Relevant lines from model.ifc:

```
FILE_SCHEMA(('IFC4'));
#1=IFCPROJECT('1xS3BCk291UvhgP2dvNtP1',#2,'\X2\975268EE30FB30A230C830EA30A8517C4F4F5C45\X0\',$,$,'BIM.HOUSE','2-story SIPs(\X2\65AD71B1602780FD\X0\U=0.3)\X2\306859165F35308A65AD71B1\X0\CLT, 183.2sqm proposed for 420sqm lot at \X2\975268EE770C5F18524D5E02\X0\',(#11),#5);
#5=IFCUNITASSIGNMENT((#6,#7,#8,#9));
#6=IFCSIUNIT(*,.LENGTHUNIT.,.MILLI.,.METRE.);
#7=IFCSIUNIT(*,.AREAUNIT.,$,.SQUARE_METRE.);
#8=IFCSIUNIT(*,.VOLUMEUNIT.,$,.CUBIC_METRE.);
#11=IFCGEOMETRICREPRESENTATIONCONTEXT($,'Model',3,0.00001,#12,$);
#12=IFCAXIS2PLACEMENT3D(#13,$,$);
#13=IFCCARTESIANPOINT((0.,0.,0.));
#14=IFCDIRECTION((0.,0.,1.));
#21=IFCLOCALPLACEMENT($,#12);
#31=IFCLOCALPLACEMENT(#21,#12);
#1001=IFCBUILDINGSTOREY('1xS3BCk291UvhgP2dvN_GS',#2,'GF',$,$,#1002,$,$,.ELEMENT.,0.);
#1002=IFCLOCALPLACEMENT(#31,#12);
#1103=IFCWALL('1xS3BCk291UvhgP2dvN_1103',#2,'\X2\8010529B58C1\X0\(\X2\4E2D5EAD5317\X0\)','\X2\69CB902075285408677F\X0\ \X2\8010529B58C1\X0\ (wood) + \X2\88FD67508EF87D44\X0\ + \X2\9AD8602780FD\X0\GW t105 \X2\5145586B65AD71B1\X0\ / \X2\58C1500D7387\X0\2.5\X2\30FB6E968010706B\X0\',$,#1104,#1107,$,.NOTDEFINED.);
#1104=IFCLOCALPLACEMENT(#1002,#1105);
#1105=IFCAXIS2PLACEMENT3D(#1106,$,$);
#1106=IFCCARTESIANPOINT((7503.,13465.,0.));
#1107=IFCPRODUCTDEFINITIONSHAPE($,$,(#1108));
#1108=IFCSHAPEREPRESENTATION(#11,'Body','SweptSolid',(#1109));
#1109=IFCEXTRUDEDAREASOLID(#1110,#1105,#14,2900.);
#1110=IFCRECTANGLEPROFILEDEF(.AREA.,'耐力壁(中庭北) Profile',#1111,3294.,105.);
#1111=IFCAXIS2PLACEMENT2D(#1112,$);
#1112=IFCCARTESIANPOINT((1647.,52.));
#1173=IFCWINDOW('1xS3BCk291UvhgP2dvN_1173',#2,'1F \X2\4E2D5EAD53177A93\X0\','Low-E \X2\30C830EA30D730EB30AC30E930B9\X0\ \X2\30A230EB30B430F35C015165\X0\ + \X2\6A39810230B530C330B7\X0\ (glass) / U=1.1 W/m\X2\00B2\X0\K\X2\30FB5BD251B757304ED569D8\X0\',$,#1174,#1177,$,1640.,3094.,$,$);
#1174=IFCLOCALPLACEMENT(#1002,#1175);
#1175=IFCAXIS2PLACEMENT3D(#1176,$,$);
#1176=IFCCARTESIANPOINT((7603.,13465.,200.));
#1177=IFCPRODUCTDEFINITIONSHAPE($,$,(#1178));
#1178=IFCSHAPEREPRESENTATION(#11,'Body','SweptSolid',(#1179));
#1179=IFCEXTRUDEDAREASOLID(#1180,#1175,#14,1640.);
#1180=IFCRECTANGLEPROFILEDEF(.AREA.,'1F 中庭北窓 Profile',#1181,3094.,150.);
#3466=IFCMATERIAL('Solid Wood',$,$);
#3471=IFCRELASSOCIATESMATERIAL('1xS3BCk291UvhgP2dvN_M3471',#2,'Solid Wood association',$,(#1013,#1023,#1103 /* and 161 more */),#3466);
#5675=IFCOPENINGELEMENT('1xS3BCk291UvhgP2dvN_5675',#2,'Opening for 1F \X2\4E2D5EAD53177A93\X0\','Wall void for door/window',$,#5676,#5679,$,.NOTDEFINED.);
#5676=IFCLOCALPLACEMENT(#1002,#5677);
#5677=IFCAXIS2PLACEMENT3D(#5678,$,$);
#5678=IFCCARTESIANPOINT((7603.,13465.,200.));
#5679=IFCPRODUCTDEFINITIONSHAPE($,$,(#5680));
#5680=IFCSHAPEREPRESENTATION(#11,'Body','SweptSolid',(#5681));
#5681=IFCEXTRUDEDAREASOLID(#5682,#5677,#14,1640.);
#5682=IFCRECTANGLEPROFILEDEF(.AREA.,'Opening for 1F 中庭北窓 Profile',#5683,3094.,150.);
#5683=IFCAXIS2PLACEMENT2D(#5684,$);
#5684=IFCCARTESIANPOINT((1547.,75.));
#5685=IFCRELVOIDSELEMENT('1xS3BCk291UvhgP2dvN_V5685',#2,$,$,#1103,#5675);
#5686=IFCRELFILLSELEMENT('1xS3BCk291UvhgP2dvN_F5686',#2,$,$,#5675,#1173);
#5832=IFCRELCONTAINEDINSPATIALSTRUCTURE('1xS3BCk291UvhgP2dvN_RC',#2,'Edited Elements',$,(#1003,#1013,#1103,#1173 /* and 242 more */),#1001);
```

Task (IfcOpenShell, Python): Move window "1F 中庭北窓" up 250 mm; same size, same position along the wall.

```python
import numpy as np
import ifcopenshell
import ifcopenshell.api.geometry
import ifcopenshell.util.placement
import ifcopenshell.util.unit

model = ifcopenshell.open("model.ifc")
unit_scale = ifcopenshell.util.unit.calculate_unit_scale(model)

window = model.by_guid("1xS3BCk291UvhgP2dvN_1173")
opening = window.FillsVoids[0].RelatingOpeningElement
dz = 250.0

shift = np.array([0.0, 0.0, dz])
# The window is not placed relative to its opening, so move both.
for product in (opening, window):
    matrix = ifcopenshell.util.placement.get_local_placement(product.ObjectPlacement)
    matrix[:3, 3] += shift
    ifcopenshell.api.geometry.edit_object_placement(model, product=product, matrix=matrix, is_si=False)

print(f"moved by {dz * unit_scale:+.3f} m")

model.write("model_v2.ifc")
```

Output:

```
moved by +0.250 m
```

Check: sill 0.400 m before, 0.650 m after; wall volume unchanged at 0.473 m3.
